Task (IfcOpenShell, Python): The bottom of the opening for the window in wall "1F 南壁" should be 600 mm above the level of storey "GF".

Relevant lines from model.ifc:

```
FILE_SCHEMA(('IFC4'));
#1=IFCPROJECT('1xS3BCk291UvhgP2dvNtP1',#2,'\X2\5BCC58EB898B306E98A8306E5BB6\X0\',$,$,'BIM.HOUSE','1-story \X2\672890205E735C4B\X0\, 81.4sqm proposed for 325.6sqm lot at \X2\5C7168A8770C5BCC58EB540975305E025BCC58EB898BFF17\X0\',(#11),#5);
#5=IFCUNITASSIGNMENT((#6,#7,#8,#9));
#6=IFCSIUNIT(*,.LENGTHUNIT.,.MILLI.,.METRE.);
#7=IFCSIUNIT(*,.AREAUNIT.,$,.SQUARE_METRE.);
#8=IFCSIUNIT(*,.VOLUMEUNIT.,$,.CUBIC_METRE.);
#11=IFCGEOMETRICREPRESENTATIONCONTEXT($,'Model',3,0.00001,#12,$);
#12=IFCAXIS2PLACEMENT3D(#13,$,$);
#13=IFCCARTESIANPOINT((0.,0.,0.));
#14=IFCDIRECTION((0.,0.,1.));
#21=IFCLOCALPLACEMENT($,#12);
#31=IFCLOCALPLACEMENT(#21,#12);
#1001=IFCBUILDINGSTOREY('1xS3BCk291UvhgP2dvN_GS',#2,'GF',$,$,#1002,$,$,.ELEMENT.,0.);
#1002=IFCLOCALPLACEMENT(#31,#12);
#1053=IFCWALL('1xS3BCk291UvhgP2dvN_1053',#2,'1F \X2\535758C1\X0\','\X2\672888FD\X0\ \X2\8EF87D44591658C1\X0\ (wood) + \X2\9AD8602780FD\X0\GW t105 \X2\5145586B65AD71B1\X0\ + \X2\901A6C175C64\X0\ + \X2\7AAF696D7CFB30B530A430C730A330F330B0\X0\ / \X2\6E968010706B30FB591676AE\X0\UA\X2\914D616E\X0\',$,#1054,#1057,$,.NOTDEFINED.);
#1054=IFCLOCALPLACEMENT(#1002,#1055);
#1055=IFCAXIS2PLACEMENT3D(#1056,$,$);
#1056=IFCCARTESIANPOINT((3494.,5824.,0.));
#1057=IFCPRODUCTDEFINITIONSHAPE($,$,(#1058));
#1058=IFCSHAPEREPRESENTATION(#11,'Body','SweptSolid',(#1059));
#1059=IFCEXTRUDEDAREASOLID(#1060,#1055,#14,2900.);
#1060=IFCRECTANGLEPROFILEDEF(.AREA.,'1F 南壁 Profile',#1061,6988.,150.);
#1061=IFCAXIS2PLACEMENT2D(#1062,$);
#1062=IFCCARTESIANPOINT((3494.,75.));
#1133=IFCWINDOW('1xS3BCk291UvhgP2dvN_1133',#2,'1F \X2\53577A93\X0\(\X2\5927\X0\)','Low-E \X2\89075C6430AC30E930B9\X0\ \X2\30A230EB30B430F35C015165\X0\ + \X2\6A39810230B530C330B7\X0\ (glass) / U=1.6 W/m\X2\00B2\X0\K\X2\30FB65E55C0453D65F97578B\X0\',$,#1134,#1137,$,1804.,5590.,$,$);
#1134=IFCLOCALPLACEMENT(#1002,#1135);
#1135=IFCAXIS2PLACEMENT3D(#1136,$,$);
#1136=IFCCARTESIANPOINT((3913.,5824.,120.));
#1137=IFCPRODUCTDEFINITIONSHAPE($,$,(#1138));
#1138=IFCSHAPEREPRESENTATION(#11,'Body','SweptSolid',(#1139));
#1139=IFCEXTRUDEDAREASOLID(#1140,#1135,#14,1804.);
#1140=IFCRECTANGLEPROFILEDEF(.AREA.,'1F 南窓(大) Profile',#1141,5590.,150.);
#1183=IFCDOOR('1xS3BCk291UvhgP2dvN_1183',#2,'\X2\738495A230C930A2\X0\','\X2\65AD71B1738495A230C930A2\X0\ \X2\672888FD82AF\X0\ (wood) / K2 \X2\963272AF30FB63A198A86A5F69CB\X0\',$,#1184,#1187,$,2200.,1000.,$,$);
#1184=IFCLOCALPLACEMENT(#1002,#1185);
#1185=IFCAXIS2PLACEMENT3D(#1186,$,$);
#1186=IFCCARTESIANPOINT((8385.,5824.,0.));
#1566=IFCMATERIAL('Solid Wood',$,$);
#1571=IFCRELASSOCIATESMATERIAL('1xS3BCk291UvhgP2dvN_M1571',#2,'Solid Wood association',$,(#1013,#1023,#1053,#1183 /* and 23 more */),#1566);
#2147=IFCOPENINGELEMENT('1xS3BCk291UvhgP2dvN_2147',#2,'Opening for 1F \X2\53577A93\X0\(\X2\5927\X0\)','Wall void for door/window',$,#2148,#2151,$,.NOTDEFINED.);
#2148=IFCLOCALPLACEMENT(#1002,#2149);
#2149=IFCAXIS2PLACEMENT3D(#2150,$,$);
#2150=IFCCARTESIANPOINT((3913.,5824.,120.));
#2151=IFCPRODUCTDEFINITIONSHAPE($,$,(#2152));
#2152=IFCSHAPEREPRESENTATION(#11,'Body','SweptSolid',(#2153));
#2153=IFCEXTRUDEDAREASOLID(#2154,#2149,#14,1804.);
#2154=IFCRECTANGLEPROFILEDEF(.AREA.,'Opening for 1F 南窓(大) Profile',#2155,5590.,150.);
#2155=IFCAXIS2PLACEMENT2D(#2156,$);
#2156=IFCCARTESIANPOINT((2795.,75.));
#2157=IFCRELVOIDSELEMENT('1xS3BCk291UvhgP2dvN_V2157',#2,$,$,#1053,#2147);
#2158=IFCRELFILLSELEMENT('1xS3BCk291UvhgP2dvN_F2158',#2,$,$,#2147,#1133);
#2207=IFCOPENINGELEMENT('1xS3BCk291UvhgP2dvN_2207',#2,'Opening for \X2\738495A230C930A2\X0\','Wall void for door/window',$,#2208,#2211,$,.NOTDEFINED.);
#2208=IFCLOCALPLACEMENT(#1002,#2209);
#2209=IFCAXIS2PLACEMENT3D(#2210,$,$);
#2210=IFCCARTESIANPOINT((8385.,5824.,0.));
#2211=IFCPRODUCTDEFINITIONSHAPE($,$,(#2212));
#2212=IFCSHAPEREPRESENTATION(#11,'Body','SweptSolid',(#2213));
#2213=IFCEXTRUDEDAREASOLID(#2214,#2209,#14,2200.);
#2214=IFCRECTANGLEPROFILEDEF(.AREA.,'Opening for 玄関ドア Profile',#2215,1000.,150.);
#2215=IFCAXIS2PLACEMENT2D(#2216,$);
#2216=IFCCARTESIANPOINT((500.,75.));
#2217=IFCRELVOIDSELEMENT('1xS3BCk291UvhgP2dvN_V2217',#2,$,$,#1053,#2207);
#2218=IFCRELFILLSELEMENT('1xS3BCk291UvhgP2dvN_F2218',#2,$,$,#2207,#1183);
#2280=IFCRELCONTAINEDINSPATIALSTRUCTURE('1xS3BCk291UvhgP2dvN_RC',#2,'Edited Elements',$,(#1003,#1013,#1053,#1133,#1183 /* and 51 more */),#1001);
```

```python
import numpy as np
import ifcopenshell
import ifcopenshell.api.geometry
import ifcopenshell.geom
import ifcopenshell.util.element
import ifcopenshell.util.placement
import ifcopenshell.util.shape
import ifcopenshell.util.unit

model = ifcopenshell.open("model.ifc")
unit_scale = ifcopenshell.util.unit.calculate_unit_scale(model)

window = model.by_guid("1xS3BCk291UvhgP2dvN_1133")
opening = window.FillsVoids[0].RelatingOpeningElement
storey = ifcopenshell.util.element.get_container(window, ifc_class="IfcBuildingStorey")
level = ifcopenshell.util.placement.get_local_placement(storey.ObjectPlacement)[2, 3]

# The opening's origin need not be at the sill, so measure its lowest point.
shape = ifcopenshell.geom.create_shape(ifcopenshell.geom.settings(), opening)
bottom = ifcopenshell.util.shape.get_shape_bottom_elevation(shape, shape.geometry) / unit_scale
dz = level + 0.6 / unit_scale - bottom

shift = np.array([0.0, 0.0, dz])
# The window is not placed relative to its opening, so move both.
for product in (opening, window):
    matrix = ifcopenshell.util.placement.get_local_placement(product.ObjectPlacement)
    matrix[:3, 3] += shift
    ifcopenshell.api.geometry.edit_object_placement(model, product=product, matrix=matrix, is_si=False)

print(f"moved by {dz * unit_scale:+.3f} m")

model.write("model_updated.ifc")
```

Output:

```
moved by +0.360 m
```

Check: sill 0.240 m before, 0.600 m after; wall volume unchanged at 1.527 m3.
